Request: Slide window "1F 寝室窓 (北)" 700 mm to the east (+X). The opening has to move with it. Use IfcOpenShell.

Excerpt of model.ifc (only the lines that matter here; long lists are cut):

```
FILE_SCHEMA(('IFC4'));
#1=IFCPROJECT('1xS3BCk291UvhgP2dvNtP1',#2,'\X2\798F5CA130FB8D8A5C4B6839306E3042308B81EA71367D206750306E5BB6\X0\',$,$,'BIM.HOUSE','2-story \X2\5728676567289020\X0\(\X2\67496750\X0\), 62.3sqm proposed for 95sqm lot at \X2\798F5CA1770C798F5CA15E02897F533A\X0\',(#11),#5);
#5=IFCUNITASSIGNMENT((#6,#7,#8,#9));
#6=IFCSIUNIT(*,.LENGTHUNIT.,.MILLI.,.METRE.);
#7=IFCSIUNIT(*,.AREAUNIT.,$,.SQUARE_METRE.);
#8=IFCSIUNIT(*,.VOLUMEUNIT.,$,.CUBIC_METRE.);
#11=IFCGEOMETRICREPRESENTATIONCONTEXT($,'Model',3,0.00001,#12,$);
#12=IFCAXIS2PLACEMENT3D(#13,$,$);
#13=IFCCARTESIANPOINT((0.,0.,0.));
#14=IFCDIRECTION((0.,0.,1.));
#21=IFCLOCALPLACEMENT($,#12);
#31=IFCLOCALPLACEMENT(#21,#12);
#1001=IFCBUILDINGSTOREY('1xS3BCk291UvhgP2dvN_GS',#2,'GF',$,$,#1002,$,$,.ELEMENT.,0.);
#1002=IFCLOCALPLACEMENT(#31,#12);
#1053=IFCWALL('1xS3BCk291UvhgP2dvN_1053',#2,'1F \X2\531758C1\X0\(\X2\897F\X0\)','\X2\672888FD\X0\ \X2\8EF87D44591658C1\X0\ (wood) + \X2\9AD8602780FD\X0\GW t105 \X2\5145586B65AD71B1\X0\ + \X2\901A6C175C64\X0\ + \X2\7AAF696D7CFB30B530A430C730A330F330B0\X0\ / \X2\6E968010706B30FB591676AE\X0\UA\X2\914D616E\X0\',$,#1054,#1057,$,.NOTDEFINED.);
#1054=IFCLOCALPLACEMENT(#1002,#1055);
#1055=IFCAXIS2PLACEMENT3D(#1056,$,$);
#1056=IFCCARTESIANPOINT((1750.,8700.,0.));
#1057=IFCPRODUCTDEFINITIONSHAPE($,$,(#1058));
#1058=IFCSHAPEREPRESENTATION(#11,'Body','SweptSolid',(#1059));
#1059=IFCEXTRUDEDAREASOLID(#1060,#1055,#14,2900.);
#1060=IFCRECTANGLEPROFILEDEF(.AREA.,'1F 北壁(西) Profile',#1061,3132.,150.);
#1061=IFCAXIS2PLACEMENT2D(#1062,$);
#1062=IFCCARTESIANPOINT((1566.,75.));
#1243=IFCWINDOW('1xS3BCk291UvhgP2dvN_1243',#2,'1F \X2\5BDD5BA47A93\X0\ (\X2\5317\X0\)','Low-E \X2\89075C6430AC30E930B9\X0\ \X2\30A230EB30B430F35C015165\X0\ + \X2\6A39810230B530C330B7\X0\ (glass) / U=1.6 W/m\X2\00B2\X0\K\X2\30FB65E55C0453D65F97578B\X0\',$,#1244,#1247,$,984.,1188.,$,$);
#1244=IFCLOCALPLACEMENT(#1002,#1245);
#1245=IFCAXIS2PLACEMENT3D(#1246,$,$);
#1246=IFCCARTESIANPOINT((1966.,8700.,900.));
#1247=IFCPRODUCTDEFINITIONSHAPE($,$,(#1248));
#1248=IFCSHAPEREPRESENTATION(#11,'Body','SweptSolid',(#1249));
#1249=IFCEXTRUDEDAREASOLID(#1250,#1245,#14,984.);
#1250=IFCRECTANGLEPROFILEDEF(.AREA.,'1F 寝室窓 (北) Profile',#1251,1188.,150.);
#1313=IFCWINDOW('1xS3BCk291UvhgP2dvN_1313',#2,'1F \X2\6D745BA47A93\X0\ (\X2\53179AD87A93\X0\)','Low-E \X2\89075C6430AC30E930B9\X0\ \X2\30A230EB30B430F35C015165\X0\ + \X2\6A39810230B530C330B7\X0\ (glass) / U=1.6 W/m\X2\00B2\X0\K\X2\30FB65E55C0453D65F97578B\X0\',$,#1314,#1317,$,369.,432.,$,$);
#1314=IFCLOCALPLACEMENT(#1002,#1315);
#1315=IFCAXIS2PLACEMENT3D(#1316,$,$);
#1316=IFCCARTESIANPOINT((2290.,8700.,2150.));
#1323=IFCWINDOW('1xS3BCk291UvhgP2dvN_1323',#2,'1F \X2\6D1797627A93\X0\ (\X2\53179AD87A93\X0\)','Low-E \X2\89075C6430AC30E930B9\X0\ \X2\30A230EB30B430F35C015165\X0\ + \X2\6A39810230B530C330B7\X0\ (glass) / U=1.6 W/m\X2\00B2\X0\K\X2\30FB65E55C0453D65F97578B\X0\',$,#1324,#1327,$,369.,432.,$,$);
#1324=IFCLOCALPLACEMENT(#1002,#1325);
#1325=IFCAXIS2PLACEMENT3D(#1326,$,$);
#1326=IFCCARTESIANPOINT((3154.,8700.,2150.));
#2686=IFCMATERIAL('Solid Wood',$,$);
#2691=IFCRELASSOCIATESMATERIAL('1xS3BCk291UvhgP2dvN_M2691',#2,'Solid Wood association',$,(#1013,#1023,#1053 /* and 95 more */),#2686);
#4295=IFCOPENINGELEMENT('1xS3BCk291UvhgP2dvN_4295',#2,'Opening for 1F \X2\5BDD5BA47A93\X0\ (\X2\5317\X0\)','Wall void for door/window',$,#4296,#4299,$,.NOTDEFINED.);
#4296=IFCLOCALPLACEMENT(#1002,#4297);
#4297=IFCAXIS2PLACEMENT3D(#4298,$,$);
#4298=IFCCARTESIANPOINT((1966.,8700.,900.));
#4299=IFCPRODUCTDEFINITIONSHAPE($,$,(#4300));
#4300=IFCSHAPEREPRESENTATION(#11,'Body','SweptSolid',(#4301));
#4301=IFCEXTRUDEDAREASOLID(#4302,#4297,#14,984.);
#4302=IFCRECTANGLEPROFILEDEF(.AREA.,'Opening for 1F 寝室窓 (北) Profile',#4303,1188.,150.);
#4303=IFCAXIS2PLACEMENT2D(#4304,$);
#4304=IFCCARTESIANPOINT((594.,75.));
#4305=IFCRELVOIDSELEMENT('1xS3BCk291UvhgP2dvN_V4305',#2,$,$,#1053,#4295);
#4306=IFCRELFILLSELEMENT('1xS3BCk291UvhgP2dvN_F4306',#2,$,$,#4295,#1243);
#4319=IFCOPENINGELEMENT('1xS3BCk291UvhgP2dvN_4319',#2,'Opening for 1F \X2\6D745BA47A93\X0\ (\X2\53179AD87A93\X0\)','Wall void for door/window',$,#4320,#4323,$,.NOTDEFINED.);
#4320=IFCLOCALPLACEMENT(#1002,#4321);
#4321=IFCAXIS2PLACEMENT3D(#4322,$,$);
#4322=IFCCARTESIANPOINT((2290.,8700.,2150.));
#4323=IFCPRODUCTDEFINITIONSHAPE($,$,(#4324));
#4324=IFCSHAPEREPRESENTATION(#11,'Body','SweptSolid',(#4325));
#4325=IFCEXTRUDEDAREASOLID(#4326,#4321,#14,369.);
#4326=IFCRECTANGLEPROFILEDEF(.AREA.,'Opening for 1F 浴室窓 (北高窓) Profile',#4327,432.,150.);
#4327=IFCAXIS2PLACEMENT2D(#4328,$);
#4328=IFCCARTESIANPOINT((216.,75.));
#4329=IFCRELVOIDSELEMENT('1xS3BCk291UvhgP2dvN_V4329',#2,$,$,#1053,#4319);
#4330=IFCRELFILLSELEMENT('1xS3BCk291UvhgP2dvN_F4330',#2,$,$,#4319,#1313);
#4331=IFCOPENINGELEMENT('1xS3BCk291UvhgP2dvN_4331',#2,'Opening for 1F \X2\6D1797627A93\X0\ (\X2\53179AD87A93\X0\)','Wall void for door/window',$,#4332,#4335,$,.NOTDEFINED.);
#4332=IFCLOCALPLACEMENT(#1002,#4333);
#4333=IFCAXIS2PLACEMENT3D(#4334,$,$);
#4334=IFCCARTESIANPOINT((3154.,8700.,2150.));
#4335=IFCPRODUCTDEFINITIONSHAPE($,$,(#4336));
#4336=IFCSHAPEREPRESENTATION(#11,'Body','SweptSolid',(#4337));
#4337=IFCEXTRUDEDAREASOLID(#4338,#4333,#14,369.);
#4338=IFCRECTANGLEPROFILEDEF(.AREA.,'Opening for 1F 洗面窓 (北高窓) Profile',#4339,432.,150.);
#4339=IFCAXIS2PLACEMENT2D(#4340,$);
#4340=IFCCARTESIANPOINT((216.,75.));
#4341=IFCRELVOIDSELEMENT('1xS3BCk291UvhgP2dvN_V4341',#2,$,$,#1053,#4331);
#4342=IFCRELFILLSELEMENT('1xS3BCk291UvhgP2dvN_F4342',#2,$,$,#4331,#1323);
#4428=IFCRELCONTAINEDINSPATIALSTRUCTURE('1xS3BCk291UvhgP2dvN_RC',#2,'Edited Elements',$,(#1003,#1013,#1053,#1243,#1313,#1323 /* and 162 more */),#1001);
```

```python
import ifcopenshell
import ifcopenshell.api.geometry
import ifcopenshell.util.placement
import ifcopenshell.util.unit

model = ifcopenshell.open("model.ifc")
unit_scale = ifcopenshell.util.unit.calculate_unit_scale(model)

window = model.by_guid("1xS3BCk291UvhgP2dvN_1243")
opening = window.FillsVoids[0].RelatingOpeningElement
wall = opening.VoidsElements[0].RelatingBuildingElement

wall_matrix = ifcopenshell.util.placement.get_local_placement(wall.ObjectPlacement)
shift = wall_matrix[:3, 0] * 0.7 / unit_scale
before = ifcopenshell.util.placement.get_local_placement(window.ObjectPlacement)[:3, 3].copy()

# The window is not placed relative to its opening, so move both.
for product in (opening, window):
    matrix = ifcopenshell.util.placement.get_local_placement(product.ObjectPlacement)
    matrix[:3, 3] += shift
    ifcopenshell.api.geometry.edit_object_placement(model, product=product, matrix=matrix, is_si=False)

after = ifcopenshell.util.placement.get_local_placement(window.ObjectPlacement)[:3, 3]
print("window moved by", (after - before).round(3) + 0.0)

model.write("model_rev.ifc")
```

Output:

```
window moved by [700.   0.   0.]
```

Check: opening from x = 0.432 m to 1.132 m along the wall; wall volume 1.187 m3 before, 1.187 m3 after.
